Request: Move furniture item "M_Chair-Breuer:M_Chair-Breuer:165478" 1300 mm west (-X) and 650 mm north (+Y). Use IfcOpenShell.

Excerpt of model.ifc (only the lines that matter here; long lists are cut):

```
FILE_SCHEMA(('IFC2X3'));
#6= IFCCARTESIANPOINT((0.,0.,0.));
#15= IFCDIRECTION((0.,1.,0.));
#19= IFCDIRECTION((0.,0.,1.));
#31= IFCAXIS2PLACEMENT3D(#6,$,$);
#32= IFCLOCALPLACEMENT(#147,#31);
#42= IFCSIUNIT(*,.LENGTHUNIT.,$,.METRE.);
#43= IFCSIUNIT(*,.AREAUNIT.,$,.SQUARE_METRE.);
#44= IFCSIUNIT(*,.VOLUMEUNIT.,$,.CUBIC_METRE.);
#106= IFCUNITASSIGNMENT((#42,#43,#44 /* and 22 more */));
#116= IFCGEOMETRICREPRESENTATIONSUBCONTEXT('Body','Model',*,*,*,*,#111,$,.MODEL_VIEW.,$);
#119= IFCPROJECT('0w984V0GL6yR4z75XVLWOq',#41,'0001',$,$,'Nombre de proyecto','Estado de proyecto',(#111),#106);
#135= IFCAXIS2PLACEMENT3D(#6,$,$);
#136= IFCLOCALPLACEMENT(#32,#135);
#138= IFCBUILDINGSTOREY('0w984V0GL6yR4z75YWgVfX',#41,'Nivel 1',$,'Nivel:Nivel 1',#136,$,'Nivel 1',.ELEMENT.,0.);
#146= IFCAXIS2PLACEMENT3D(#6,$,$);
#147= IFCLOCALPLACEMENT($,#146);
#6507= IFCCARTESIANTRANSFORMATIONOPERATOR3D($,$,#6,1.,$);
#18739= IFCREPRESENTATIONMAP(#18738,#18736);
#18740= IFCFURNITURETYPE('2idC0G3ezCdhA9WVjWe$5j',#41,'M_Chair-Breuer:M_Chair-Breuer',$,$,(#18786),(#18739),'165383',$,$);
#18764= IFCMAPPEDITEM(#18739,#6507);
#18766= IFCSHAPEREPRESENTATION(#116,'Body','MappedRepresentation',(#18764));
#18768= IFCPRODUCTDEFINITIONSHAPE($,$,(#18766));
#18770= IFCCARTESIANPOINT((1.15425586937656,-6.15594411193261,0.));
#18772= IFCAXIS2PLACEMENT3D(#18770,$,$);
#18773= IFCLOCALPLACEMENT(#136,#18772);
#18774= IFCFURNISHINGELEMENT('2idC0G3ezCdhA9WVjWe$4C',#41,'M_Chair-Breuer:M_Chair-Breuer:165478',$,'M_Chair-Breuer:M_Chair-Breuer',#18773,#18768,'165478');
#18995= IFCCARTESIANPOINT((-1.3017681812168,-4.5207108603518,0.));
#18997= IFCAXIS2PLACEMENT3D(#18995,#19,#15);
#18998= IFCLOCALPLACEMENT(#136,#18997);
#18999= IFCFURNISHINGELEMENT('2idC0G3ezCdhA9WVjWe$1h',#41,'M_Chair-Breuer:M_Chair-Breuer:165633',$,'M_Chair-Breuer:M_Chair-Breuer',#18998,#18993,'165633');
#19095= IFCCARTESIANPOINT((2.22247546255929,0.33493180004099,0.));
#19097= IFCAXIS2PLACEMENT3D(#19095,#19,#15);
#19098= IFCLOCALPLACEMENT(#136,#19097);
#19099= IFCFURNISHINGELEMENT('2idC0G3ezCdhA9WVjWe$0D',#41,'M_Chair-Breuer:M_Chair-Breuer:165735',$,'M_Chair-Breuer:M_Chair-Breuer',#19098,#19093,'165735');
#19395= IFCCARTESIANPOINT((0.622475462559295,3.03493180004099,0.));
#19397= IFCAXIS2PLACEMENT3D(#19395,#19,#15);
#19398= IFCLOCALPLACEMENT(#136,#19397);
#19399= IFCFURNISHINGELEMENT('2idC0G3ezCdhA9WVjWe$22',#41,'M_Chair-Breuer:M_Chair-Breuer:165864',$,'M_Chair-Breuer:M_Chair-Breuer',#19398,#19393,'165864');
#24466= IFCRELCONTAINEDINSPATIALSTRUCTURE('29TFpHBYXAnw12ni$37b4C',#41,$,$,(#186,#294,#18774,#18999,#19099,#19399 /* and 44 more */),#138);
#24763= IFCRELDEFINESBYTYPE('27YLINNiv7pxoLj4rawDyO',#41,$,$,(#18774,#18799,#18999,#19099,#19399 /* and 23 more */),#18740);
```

```python
import ifcopenshell
import ifcopenshell.api.geometry
import ifcopenshell.util.placement

model = ifcopenshell.open("model.ifc")

item = model.by_id(18774)
matrix = ifcopenshell.util.placement.get_local_placement(item.ObjectPlacement)
matrix[0, 3] -= 1.3
matrix[1, 3] += 0.65
ifcopenshell.api.geometry.edit_object_placement(model, product=item, matrix=matrix, is_si=False)

print(ifcopenshell.util.placement.get_local_placement(item.ObjectPlacement).round(3) + 0.0)

model.write("model_rev.ifc")
```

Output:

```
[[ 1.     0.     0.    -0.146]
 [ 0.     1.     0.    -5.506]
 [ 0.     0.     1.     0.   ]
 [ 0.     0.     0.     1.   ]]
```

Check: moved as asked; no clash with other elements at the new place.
